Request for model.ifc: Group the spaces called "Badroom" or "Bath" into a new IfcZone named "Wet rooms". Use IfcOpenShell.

First a look at what the model holds.

```python
import ifcopenshell

model = ifcopenshell.open("model.ifc")
print(model.schema)
seen = {}
for space in model.by_type("IfcSpace"):
    seen[space.LongName] = seen.get(space.LongName, 0) + 1
for name, count in sorted(seen.items(), key=str):
    print(count, "x", name)
print("zones:", [z.Name for z in model.by_type("IfcZone")][:20])
```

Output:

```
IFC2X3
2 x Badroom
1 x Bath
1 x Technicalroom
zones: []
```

```python
import ifcopenshell
import ifcopenshell.api.group
import ifcopenshell.api.root

model = ifcopenshell.open("model.ifc")

names = {"Badroom", "Bath"}
spaces = [s for s in model.by_type("IfcSpace") if s.LongName in names]

zone = ifcopenshell.api.root.create_entity(model, ifc_class="IfcZone", name="Wet rooms")
ifcopenshell.api.group.assign_group(model, products=spaces, group=zone)
print(len(spaces), "spaces in", zone.Name)

model.write("model-out.ifc")
```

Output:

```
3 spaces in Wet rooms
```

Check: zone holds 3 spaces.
